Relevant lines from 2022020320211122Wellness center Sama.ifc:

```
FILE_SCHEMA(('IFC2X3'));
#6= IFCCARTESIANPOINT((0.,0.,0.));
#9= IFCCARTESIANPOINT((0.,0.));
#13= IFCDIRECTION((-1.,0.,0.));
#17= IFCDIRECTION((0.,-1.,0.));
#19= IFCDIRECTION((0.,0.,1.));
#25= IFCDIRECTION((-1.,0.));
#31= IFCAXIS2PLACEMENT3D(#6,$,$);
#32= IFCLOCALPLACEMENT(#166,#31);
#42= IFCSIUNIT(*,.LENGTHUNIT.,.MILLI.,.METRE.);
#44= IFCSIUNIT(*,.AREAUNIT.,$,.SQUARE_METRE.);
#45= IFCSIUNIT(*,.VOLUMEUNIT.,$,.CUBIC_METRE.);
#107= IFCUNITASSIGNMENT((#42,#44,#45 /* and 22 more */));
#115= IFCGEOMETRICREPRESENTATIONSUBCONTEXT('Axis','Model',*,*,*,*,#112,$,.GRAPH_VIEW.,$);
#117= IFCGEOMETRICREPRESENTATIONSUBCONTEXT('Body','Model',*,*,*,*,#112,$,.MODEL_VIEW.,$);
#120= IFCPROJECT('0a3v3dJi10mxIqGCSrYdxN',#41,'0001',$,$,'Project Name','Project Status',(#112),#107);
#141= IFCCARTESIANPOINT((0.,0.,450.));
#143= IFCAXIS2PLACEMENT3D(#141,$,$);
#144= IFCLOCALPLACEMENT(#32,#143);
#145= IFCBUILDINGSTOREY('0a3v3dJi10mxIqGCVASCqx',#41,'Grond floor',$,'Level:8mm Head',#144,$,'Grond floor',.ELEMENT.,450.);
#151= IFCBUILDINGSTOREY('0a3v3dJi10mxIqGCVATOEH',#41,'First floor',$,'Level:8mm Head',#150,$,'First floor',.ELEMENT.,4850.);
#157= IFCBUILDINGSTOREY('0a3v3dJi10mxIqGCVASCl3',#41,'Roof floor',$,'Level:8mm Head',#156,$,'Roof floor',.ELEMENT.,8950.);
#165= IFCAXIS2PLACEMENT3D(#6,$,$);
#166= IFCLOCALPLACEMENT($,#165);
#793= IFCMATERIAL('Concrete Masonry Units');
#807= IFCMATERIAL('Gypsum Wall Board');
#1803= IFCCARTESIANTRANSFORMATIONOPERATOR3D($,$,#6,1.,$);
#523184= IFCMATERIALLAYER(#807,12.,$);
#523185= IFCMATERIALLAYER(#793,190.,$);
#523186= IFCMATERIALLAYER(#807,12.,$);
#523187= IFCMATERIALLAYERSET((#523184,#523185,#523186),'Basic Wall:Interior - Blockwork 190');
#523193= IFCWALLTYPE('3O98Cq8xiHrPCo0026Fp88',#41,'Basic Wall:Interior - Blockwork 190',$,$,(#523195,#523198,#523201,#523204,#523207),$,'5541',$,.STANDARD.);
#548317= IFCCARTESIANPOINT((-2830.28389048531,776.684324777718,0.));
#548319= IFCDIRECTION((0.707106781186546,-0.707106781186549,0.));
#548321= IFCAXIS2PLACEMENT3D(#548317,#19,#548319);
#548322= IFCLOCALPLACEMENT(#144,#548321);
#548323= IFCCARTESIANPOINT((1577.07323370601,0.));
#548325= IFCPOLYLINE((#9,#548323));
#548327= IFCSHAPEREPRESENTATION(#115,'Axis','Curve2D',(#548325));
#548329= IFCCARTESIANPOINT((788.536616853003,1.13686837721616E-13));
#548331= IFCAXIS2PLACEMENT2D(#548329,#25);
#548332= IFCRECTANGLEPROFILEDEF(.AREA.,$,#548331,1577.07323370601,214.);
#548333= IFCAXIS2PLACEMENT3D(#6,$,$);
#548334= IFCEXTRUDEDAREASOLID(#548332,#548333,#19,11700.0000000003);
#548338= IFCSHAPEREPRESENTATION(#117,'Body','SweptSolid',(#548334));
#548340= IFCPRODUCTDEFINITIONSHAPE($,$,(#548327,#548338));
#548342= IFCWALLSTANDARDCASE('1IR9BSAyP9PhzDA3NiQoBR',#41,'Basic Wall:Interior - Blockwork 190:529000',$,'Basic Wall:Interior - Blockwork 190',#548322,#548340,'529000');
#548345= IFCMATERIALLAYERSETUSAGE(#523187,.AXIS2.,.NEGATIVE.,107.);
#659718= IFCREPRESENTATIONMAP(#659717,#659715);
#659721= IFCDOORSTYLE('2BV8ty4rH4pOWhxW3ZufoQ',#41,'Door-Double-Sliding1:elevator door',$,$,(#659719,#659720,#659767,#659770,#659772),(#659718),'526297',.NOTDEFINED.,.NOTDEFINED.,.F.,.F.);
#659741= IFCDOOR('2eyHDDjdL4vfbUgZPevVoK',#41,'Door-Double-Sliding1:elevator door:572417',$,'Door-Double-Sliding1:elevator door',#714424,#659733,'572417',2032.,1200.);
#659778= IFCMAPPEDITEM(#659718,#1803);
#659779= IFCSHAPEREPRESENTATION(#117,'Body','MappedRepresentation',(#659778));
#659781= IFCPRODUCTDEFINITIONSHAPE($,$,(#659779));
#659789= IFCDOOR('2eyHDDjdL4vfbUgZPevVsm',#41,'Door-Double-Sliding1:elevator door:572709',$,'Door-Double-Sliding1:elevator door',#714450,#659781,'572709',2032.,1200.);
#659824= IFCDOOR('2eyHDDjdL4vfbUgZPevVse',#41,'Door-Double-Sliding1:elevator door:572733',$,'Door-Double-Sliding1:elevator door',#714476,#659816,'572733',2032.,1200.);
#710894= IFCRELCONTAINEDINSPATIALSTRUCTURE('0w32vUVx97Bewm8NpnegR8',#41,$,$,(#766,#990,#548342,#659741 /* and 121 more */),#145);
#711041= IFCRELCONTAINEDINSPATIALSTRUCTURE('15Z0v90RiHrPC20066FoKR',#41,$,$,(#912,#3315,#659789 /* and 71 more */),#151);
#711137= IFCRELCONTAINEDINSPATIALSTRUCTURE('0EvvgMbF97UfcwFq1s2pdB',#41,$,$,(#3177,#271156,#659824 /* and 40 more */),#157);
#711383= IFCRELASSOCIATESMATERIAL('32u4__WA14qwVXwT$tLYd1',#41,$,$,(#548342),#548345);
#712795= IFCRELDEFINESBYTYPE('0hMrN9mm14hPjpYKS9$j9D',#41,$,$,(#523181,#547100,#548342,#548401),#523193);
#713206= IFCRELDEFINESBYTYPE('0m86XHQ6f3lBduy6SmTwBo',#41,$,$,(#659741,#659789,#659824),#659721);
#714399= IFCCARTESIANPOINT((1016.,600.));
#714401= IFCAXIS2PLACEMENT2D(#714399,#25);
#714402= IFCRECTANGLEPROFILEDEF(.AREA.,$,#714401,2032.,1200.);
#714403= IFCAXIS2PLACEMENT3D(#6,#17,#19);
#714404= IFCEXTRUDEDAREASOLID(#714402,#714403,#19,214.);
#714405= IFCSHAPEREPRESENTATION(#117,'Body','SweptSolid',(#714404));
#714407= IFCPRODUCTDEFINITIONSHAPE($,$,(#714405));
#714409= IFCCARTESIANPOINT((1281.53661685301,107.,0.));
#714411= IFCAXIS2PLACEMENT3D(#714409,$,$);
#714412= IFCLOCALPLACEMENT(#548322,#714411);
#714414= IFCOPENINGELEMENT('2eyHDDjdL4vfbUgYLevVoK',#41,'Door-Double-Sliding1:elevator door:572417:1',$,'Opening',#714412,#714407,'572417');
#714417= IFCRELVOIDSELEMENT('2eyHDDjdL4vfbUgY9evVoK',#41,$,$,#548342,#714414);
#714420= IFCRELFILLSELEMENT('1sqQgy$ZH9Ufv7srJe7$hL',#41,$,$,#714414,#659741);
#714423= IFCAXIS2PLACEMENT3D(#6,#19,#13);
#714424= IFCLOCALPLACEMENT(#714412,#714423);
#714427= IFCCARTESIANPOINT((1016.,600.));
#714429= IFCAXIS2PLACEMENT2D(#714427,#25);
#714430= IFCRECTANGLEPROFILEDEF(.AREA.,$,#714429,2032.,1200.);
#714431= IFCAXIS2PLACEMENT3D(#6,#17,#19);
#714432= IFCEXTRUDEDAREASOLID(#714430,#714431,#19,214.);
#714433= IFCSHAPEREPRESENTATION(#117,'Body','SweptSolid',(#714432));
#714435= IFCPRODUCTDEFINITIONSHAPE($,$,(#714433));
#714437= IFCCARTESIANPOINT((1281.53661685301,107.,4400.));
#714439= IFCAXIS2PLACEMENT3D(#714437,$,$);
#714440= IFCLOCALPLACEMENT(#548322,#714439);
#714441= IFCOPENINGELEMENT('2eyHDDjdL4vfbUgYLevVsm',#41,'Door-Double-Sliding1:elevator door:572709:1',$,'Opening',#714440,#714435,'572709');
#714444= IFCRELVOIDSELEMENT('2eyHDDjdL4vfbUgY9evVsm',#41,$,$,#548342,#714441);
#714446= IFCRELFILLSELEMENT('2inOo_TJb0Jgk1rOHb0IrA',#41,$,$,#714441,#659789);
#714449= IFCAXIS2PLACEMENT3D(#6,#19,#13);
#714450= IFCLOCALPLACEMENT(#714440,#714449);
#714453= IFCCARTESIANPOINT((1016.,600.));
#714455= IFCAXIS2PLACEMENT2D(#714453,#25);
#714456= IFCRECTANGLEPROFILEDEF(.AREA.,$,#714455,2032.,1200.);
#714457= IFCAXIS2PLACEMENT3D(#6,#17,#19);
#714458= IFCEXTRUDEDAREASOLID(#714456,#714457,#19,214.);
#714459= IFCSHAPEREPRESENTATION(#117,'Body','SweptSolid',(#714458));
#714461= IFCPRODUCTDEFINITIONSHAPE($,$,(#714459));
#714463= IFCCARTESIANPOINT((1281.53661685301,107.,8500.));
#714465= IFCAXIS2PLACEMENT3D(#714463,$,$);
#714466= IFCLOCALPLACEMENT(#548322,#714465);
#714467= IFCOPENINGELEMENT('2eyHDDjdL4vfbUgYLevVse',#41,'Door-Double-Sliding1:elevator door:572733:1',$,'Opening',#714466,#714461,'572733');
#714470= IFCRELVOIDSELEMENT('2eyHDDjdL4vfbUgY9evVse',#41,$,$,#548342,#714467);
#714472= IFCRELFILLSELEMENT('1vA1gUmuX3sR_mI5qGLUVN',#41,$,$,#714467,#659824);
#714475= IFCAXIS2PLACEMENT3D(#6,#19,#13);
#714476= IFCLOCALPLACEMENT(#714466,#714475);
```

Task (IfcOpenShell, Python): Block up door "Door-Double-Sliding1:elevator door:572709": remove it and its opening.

```python
import ifcopenshell
import ifcopenshell.api.feature
import ifcopenshell.api.root
import ifcopenshell.geom
import ifcopenshell.util.shape

model = ifcopenshell.open("2022020320211122Wellness center Sama.ifc")
settings = ifcopenshell.geom.settings()


def volume(element):
    """Net volume in cubic metres, openings subtracted."""
    shape = ifcopenshell.geom.create_shape(settings, element)
    return ifcopenshell.util.shape.get_volume(shape.geometry)


door = model.by_guid("2eyHDDjdL4vfbUgZPevVsm")
opening = door.FillsVoids[0].RelatingOpeningElement
wall = opening.VoidsElements[0].RelatingBuildingElement
before = volume(wall)

ifcopenshell.api.root.remove_product(model, product=door)
ifcopenshell.api.feature.remove_feature(model, feature=opening)

after = volume(wall)

print(f"wall volume {before:.3f} -> {after:.3f} m3")

model.write("2022020320211122Wellness center Sama_v2.ifc")
```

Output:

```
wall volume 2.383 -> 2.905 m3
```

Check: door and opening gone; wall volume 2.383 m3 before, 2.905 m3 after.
